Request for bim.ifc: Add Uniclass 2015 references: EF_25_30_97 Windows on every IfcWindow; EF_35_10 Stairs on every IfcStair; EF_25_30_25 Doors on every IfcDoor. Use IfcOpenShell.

First a look at what the model holds.

```python
import ifcopenshell

model = ifcopenshell.open("bim.ifc")
print(model.schema)
print("classifications:", [c.Name for c in model.by_type("IfcClassification")])
for ifc_class in ("IfcDoor", "IfcRoof", "IfcStair", "IfcWall", "IfcWindow"):
    print(ifc_class, len(model.by_type(ifc_class)))
```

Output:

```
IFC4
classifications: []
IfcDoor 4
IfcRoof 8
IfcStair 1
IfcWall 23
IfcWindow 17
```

```python
import ifcopenshell
import ifcopenshell.api.classification

model = ifcopenshell.open("bim.ifc")

system = ifcopenshell.api.classification.add_classification(model, classification="Uniclass 2015")

codes = {
    "IfcWindow": ("EF_25_30_97", "Windows"),
    "IfcStair": ("EF_35_10", "Stairs"),
    "IfcDoor": ("EF_25_30_25", "Doors"),
}
for ifc_class, (code, name) in codes.items():
    products = model.by_type(ifc_class)
    ifcopenshell.api.classification.add_reference(
        model, products=products, classification=system, identification=code, name=name
    )
    print(code, len(products))

model.write("bim-out.ifc")
```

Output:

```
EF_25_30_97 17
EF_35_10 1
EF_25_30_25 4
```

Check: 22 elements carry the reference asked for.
